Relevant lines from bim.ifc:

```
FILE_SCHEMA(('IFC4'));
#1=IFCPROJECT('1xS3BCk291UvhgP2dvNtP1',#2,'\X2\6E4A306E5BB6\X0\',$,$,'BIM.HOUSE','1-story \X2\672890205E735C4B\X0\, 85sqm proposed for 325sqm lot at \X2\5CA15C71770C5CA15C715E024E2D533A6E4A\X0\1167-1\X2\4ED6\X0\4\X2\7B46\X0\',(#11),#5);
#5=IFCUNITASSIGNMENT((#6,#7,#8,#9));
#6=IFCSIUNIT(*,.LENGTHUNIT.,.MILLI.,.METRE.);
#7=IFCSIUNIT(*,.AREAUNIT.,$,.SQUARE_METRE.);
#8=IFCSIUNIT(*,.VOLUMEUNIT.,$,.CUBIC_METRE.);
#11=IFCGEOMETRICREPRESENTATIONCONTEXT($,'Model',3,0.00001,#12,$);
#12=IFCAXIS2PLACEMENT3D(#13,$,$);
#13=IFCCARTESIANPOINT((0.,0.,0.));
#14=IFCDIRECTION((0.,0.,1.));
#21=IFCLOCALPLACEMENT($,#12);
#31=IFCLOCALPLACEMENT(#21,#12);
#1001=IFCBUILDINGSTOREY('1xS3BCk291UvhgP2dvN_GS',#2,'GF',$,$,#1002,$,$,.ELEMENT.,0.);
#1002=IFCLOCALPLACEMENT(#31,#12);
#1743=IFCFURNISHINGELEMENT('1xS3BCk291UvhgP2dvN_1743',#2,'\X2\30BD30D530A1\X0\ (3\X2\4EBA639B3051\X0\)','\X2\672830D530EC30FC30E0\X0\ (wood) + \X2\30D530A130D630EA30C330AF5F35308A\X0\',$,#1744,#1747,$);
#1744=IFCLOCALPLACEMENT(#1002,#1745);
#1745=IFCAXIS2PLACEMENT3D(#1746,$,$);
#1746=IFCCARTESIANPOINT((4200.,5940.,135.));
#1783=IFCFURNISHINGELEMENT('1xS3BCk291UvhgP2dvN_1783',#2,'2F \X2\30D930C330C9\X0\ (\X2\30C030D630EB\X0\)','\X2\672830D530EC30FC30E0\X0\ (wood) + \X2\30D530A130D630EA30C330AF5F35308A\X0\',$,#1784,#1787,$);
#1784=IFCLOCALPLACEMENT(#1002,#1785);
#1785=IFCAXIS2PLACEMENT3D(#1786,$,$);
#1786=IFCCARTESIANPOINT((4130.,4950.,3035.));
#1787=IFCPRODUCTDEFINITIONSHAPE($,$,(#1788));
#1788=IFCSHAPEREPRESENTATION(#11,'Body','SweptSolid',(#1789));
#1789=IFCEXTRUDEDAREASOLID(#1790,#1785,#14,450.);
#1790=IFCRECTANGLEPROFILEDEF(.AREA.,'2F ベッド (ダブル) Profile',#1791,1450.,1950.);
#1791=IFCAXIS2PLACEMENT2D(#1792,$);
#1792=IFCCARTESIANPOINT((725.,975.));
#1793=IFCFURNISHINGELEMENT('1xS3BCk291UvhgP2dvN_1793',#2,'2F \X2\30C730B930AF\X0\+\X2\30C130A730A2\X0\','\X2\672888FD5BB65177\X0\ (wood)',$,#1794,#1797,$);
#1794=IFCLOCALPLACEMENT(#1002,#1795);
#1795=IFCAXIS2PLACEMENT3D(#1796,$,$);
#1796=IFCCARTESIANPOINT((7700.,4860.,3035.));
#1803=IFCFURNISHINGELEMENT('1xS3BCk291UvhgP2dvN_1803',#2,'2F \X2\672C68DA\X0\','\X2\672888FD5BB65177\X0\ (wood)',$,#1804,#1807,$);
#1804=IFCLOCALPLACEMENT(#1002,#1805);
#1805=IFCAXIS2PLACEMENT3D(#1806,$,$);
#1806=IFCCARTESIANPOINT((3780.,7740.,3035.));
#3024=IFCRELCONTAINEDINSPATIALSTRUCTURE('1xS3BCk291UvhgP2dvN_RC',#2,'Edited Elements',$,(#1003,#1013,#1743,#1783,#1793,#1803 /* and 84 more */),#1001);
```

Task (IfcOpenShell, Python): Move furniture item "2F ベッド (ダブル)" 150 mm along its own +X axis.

```python
import ifcopenshell
import ifcopenshell.api.geometry
import ifcopenshell.util.placement
import ifcopenshell.util.unit

model = ifcopenshell.open("bim.ifc")
unit_scale = ifcopenshell.util.unit.calculate_unit_scale(model)

item = model.by_id(1783)
matrix = ifcopenshell.util.placement.get_local_placement(item.ObjectPlacement)
matrix[:3, 3] += matrix[:3, 0] * 0.15 / unit_scale
ifcopenshell.api.geometry.edit_object_placement(model, product=item, matrix=matrix, is_si=False)

print(ifcopenshell.util.placement.get_local_placement(item.ObjectPlacement).round(3) + 0.0)

model.write("bim_v2.ifc")
```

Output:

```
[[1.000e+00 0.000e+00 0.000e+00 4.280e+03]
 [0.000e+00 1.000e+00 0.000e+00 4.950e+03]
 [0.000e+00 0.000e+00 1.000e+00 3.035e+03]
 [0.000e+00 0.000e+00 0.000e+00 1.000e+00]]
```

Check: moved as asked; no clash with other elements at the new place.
